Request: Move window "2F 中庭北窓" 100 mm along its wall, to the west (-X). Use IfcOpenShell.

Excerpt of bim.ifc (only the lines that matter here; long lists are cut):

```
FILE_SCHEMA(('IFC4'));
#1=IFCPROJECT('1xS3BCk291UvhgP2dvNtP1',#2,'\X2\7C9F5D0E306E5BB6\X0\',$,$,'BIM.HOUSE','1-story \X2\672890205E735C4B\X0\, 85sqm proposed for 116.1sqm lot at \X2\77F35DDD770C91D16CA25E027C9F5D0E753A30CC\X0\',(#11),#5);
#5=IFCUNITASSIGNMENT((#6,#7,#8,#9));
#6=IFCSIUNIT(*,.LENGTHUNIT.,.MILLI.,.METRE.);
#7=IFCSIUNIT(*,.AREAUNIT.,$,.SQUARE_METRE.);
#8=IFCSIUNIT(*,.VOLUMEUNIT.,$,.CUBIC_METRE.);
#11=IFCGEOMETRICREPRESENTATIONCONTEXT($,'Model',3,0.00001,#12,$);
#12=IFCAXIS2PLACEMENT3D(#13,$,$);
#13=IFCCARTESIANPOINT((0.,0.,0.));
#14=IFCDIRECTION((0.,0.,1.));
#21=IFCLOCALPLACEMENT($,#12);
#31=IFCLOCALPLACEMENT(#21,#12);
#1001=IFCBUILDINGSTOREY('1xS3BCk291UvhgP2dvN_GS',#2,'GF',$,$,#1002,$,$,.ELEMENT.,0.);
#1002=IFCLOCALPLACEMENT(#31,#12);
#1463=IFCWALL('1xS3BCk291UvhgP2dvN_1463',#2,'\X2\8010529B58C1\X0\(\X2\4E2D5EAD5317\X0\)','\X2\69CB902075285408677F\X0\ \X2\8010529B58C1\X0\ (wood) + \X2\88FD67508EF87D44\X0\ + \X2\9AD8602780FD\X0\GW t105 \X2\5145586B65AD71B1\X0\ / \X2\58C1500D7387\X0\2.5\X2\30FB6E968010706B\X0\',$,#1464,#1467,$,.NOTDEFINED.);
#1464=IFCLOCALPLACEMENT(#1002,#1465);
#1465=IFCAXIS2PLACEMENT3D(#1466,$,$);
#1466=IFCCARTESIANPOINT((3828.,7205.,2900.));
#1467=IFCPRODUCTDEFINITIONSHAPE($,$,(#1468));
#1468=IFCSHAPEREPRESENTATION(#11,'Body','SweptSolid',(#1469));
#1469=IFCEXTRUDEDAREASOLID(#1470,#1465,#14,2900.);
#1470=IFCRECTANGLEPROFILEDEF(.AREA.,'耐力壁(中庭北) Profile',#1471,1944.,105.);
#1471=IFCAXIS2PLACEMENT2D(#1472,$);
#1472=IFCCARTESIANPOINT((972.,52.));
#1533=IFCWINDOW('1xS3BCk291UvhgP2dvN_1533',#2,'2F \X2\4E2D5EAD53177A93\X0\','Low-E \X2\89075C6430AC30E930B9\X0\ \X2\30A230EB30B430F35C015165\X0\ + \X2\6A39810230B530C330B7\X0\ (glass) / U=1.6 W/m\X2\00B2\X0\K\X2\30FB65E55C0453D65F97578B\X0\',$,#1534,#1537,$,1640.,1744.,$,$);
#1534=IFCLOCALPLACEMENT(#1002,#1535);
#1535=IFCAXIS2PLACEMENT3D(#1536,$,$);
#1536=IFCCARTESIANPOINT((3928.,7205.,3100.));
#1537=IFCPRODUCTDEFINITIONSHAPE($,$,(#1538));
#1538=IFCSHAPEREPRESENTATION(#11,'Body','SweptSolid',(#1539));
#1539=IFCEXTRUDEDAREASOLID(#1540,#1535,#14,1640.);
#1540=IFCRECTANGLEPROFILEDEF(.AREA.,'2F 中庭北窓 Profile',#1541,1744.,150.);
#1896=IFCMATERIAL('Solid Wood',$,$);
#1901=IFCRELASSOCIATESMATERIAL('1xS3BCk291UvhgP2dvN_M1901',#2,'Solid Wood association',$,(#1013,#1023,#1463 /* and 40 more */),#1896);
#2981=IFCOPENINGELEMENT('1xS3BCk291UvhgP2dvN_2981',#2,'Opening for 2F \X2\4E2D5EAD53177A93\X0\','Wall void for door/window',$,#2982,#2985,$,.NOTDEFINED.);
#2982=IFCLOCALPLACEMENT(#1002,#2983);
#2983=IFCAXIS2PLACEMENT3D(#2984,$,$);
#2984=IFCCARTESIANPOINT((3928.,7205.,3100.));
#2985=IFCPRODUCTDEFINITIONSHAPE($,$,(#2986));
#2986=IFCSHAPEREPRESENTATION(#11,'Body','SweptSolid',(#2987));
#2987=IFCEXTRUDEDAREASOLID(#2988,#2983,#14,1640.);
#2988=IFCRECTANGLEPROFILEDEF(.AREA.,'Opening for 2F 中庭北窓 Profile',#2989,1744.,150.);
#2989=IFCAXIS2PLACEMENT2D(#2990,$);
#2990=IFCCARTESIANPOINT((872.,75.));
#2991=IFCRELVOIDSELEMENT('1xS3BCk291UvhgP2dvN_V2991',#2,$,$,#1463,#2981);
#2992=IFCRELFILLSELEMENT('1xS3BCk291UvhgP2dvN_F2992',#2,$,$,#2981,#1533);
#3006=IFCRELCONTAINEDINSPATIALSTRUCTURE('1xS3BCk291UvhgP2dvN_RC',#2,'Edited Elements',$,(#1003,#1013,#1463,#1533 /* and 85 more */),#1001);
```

```python
import ifcopenshell
import ifcopenshell.api.geometry
import ifcopenshell.util.placement

model = ifcopenshell.open("bim.ifc")

window = model.by_id(1533)
opening = window.FillsVoids[0].RelatingOpeningElement
wall = opening.VoidsElements[0].RelatingBuildingElement

wall_matrix = ifcopenshell.util.placement.get_local_placement(wall.ObjectPlacement)
shift = wall_matrix[:3, 0] * -100.0
before = ifcopenshell.util.placement.get_local_placement(window.ObjectPlacement)[:3, 3].copy()

# The window is not placed relative to its opening, so move both.
for product in (opening, window):
    matrix = ifcopenshell.util.placement.get_local_placement(product.ObjectPlacement)
    matrix[:3, 3] += shift
    ifcopenshell.api.geometry.edit_object_placement(model, product=product, matrix=matrix, is_si=False)

after = ifcopenshell.util.placement.get_local_placement(window.ObjectPlacement)[:3, 3]
print("window moved by", (after - before).round(3) + 0.0)

model.write("bim-out.ifc")
```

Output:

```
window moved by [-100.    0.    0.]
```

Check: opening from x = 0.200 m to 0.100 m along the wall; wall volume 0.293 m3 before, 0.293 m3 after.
